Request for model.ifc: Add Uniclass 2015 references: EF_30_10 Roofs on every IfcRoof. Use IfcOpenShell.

First a look at what the model holds.

```python
import ifcopenshell

model = ifcopenshell.open("model.ifc")
print(model.schema)
print("classifications:", [c.Name for c in model.by_type("IfcClassification")])
for ifc_class in ("IfcDoor", "IfcRoof", "IfcStair", "IfcWall", "IfcWindow"):
    print(ifc_class, len(model.by_type(ifc_class)))
```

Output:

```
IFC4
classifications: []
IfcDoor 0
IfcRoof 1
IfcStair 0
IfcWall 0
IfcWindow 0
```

```python
import ifcopenshell
import ifcopenshell.api.classification

model = ifcopenshell.open("model.ifc")

system = ifcopenshell.api.classification.add_classification(model, classification="Uniclass 2015")

codes = {
    "IfcRoof": ("EF_30_10", "Roofs"),
}
for ifc_class, (code, name) in codes.items():
    products = model.by_type(ifc_class)
    ifcopenshell.api.classification.add_reference(
        model, products=products, classification=system, identification=code, name=name
    )
    print(code, len(products))

model.write("model_v2.ifc")
```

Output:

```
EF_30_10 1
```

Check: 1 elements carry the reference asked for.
